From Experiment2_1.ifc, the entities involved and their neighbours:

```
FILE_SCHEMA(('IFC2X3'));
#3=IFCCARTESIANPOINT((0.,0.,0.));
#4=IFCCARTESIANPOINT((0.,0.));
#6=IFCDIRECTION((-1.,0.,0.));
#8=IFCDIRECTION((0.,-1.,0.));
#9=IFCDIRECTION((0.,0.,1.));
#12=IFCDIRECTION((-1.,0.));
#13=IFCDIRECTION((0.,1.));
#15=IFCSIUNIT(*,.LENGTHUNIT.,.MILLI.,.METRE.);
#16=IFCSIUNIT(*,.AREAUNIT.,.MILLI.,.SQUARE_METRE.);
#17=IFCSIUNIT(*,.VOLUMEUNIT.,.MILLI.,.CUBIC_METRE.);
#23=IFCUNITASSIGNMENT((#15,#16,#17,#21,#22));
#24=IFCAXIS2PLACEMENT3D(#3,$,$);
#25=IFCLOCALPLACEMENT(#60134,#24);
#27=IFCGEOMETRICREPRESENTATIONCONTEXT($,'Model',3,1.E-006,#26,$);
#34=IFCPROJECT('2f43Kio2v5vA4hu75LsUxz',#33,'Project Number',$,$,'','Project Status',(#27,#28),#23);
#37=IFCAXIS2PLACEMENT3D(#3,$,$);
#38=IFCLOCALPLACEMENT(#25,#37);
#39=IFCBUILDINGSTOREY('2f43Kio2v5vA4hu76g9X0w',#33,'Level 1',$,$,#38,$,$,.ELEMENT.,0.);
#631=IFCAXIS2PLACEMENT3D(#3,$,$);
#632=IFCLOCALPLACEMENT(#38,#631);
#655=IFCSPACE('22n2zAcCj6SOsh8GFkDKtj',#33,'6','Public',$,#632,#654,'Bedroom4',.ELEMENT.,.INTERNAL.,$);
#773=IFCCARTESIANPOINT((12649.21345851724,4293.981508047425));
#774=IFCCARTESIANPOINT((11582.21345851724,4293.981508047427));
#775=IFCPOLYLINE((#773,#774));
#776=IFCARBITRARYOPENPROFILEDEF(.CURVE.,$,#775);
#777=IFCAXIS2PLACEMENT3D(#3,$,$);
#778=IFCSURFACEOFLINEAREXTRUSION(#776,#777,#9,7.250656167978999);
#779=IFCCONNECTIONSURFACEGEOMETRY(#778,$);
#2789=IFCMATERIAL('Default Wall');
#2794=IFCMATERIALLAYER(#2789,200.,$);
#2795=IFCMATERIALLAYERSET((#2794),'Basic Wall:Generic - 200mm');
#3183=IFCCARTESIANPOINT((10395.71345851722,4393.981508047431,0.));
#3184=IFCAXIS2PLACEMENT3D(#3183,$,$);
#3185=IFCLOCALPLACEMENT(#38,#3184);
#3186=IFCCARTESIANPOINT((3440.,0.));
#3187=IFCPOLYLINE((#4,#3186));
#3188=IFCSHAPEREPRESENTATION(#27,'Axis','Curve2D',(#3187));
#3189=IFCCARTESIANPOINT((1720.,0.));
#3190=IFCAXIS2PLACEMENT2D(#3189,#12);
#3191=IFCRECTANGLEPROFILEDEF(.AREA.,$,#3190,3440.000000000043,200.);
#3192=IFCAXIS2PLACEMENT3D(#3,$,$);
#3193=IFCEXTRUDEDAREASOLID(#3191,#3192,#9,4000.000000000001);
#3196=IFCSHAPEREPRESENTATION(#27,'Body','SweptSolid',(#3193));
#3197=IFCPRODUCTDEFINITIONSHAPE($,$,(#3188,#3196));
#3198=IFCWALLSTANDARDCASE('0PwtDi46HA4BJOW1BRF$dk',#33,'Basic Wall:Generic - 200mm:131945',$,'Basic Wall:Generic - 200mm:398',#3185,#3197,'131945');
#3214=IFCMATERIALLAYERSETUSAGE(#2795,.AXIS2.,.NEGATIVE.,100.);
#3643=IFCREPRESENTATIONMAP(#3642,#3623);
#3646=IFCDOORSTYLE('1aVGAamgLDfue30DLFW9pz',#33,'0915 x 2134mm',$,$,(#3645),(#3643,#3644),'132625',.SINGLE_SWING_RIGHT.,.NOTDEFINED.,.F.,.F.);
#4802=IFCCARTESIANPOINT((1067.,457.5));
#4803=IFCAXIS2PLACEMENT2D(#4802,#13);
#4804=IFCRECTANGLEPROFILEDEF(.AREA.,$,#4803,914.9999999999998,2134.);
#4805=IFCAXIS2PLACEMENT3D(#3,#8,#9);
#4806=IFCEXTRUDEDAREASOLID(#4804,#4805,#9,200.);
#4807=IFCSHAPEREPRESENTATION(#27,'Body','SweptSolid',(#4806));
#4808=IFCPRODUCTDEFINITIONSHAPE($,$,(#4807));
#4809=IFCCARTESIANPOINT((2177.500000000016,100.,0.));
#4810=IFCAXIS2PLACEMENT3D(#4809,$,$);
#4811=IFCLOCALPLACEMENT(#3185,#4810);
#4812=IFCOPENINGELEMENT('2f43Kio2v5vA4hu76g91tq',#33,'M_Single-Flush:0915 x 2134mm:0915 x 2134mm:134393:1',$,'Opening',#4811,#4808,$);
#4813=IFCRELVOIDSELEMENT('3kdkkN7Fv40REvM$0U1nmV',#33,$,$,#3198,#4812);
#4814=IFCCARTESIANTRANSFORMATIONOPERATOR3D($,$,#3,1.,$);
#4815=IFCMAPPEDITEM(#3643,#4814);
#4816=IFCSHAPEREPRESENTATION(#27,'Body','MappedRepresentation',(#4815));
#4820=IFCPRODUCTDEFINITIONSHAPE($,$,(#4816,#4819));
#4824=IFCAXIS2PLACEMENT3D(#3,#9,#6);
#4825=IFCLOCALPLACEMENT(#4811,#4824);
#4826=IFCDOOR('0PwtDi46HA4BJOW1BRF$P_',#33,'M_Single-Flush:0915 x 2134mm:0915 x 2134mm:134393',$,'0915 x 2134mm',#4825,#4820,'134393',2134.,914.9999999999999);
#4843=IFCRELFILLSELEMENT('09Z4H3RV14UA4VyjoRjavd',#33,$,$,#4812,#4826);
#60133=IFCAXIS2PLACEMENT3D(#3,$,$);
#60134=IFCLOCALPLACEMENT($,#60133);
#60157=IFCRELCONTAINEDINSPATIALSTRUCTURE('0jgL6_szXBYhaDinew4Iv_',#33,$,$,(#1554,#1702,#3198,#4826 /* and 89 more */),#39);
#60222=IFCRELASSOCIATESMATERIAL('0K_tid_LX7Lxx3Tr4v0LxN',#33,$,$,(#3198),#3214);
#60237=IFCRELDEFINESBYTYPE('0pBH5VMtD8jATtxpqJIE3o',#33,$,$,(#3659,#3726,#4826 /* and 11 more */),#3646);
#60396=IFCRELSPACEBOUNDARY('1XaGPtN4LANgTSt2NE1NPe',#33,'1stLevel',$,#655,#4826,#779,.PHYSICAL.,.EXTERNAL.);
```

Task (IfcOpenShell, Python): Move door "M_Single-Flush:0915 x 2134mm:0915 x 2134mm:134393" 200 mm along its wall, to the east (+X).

```python
import numpy as np
import ifcopenshell
import ifcopenshell.api.geometry
import ifcopenshell.util.placement

model = ifcopenshell.open("Experiment2_1.ifc")

door = model.by_guid("0PwtDi46HA4BJOW1BRF$P_")
opening = door.FillsVoids[0].RelatingOpeningElement
wall = opening.VoidsElements[0].RelatingBuildingElement

wall_matrix = ifcopenshell.util.placement.get_local_placement(wall.ObjectPlacement)
shift = wall_matrix[:3, 0] * 200.0
before = ifcopenshell.util.placement.get_local_placement(door.ObjectPlacement)[:3, 3].copy()

# The door is placed relative to its opening, so it follows when the opening moves.
matrix = ifcopenshell.util.placement.get_local_placement(opening.ObjectPlacement)
matrix[:3, 3] += shift
ifcopenshell.api.geometry.edit_object_placement(
    model, product=opening, matrix=matrix, is_si=False, should_transform_children=True
)

# Space boundary surfaces are stored in each space's coordinates; move them too.
for rel in door.ProvidesBoundaries:
    if not rel.ConnectionGeometry:
        continue
    surface = rel.ConnectionGeometry.SurfaceOnRelatingElement
    space_matrix = ifcopenshell.util.placement.get_local_placement(rel.RelatingSpace.ObjectPlacement)
    point = np.array(surface.Position.Location.Coordinates) + space_matrix[:3, :3].T @ shift
    surface.Position = model.createIfcAxis2Placement3D(
        model.createIfcCartesianPoint(point.tolist()), surface.Position.Axis, surface.Position.RefDirection
    )

after = ifcopenshell.util.placement.get_local_placement(door.ObjectPlacement)[:3, 3]
print("door moved by", (after - before).round(3) + 0.0)

model.write("Experiment2_1_rev.ifc")
```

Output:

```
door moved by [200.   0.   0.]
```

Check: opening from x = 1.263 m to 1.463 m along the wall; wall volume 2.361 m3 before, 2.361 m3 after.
